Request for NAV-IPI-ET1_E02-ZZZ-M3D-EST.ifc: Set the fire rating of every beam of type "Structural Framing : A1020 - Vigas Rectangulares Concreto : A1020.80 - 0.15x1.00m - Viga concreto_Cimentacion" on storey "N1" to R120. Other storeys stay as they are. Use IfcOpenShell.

First a look at what the model holds.

```python
import ifcopenshell
import ifcopenshell.util.element

model = ifcopenshell.open("NAV-IPI-ET1_E02-ZZZ-M3D-EST.ifc")
print(model.schema)
storey = next(s for s in model.by_type("IfcBuildingStorey") if s.Name == "N1")
beams = [e for e in ifcopenshell.util.element.get_decomposition(storey) if e.is_a("IfcBeam")]
seen = {}
for e in beams:
    element_type = ifcopenshell.util.element.get_type(e)
    key = (element_type.Name if element_type != e and element_type else None, ifcopenshell.util.element.get_pset(e, "Pset_BeamCommon", "FireRating"))
    seen[key] = seen.get(key, 0) + 1
for (name, value), count in sorted(seen.items(), key=str):
    print(count, "x", name, "|", value)
```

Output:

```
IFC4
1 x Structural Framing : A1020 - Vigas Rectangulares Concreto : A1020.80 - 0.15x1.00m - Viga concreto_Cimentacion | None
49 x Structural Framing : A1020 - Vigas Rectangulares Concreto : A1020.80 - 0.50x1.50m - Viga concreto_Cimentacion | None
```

```python
import ifcopenshell
import ifcopenshell.api.pset
import ifcopenshell.util.element

model = ifcopenshell.open("NAV-IPI-ET1_E02-ZZZ-M3D-EST.ifc")

storey = next(s for s in model.by_type("IfcBuildingStorey") if s.Name == "N1")
beams = [e for e in ifcopenshell.util.element.get_decomposition(storey) if e.is_a("IfcBeam")]

count = 0
for e in beams:
    element_type = ifcopenshell.util.element.get_type(e)
    if element_type in (None, e) or element_type.Name != "Structural Framing : A1020 - Vigas Rectangulares Concreto : A1020.80 - 0.15x1.00m - Viga concreto_Cimentacion":
        continue
    # add_pset returns the element's existing set when there is one.
    pset = ifcopenshell.api.pset.add_pset(model, product=e, name="Pset_BeamCommon")
    ifcopenshell.api.pset.edit_pset(model, pset=pset, properties={"FireRating": "R120"})
    count += 1

print(count, "beams updated")

model.write("NAV-IPI-ET1_E02-ZZZ-M3D-EST-out.ifc")
```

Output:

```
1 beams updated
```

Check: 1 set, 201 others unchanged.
